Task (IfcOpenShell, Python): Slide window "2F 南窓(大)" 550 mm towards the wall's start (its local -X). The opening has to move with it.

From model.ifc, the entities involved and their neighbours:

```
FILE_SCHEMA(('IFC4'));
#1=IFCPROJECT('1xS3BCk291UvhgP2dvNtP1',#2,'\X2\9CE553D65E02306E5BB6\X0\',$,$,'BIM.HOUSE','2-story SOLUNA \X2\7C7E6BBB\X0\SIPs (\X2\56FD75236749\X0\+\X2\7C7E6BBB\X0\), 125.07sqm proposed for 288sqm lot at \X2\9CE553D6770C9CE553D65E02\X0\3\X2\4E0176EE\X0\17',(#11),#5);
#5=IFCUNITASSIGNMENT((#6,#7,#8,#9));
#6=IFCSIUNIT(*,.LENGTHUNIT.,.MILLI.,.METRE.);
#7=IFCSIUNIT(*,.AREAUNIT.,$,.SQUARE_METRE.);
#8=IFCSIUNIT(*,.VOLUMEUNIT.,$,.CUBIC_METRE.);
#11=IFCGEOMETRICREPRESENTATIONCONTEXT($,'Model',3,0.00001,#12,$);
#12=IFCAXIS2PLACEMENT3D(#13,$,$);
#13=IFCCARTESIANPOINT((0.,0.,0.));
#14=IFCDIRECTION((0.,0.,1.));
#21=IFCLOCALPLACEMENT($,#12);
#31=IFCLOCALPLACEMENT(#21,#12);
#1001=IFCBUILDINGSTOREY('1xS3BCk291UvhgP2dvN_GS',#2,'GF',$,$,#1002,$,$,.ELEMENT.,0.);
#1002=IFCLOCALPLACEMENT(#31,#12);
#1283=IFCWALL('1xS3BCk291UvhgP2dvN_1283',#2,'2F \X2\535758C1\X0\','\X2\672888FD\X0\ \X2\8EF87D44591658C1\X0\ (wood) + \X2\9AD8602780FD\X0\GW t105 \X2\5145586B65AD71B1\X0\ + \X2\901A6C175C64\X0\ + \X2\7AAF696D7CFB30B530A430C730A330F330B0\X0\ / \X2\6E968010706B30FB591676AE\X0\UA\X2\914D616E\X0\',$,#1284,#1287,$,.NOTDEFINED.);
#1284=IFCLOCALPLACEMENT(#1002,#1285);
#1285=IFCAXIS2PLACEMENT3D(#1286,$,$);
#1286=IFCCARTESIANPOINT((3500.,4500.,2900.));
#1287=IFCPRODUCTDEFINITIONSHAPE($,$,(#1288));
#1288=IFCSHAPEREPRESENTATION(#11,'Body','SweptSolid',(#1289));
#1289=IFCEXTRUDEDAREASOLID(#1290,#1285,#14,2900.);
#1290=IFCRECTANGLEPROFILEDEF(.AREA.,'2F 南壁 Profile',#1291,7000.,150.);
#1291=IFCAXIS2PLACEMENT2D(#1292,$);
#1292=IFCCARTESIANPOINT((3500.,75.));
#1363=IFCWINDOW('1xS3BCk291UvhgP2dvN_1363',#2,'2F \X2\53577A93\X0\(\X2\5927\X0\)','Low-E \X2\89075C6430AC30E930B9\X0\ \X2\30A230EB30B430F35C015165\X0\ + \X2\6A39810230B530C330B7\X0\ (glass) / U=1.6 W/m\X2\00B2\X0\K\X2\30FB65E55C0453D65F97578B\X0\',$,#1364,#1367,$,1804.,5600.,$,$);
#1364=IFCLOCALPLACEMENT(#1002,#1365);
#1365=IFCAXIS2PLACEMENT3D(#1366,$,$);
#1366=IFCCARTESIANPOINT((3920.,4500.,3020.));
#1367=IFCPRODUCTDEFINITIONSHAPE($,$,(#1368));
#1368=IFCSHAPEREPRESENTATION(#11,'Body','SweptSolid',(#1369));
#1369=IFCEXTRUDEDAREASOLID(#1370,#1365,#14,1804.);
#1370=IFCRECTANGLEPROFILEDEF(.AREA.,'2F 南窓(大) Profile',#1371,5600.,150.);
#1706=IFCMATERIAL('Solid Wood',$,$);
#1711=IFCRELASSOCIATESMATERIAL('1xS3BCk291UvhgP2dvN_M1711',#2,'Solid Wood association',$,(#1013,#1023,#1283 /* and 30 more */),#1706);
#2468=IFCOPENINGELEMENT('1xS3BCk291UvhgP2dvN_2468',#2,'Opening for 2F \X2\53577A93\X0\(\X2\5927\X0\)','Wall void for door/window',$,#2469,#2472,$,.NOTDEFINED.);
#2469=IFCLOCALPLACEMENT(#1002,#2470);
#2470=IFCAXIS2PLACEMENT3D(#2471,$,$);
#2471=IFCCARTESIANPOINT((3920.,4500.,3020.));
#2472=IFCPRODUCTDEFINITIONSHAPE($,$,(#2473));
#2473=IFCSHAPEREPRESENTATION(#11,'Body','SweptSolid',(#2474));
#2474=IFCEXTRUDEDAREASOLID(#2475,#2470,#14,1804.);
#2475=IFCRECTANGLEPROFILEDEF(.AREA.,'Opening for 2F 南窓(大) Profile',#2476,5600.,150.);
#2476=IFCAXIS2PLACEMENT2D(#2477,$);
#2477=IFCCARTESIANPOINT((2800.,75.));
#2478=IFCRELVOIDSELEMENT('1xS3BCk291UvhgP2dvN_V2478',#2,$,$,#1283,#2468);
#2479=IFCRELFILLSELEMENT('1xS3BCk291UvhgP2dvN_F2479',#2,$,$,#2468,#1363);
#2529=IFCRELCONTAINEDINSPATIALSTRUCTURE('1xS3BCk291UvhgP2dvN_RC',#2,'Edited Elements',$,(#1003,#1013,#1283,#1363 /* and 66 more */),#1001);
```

```python
import ifcopenshell
import ifcopenshell.api.geometry
import ifcopenshell.util.placement

model = ifcopenshell.open("model.ifc")

window = model.by_guid("1xS3BCk291UvhgP2dvN_1363")
opening = window.FillsVoids[0].RelatingOpeningElement
wall = opening.VoidsElements[0].RelatingBuildingElement

wall_matrix = ifcopenshell.util.placement.get_local_placement(wall.ObjectPlacement)
shift = wall_matrix[:3, 0] * -550.0
before = ifcopenshell.util.placement.get_local_placement(window.ObjectPlacement)[:3, 3].copy()

# The window is not placed relative to its opening, so move both.
for product in (opening, window):
    matrix = ifcopenshell.util.placement.get_local_placement(product.ObjectPlacement)
    matrix[:3, 3] += shift
    ifcopenshell.api.geometry.edit_object_placement(model, product=product, matrix=matrix, is_si=False)

after = ifcopenshell.util.placement.get_local_placement(window.ObjectPlacement)[:3, 3]
print("window moved by", (after - before).round(3) + 0.0)

model.write("model_v2.ifc")
```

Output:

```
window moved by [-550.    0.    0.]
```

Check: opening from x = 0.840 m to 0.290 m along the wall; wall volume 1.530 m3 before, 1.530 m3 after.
